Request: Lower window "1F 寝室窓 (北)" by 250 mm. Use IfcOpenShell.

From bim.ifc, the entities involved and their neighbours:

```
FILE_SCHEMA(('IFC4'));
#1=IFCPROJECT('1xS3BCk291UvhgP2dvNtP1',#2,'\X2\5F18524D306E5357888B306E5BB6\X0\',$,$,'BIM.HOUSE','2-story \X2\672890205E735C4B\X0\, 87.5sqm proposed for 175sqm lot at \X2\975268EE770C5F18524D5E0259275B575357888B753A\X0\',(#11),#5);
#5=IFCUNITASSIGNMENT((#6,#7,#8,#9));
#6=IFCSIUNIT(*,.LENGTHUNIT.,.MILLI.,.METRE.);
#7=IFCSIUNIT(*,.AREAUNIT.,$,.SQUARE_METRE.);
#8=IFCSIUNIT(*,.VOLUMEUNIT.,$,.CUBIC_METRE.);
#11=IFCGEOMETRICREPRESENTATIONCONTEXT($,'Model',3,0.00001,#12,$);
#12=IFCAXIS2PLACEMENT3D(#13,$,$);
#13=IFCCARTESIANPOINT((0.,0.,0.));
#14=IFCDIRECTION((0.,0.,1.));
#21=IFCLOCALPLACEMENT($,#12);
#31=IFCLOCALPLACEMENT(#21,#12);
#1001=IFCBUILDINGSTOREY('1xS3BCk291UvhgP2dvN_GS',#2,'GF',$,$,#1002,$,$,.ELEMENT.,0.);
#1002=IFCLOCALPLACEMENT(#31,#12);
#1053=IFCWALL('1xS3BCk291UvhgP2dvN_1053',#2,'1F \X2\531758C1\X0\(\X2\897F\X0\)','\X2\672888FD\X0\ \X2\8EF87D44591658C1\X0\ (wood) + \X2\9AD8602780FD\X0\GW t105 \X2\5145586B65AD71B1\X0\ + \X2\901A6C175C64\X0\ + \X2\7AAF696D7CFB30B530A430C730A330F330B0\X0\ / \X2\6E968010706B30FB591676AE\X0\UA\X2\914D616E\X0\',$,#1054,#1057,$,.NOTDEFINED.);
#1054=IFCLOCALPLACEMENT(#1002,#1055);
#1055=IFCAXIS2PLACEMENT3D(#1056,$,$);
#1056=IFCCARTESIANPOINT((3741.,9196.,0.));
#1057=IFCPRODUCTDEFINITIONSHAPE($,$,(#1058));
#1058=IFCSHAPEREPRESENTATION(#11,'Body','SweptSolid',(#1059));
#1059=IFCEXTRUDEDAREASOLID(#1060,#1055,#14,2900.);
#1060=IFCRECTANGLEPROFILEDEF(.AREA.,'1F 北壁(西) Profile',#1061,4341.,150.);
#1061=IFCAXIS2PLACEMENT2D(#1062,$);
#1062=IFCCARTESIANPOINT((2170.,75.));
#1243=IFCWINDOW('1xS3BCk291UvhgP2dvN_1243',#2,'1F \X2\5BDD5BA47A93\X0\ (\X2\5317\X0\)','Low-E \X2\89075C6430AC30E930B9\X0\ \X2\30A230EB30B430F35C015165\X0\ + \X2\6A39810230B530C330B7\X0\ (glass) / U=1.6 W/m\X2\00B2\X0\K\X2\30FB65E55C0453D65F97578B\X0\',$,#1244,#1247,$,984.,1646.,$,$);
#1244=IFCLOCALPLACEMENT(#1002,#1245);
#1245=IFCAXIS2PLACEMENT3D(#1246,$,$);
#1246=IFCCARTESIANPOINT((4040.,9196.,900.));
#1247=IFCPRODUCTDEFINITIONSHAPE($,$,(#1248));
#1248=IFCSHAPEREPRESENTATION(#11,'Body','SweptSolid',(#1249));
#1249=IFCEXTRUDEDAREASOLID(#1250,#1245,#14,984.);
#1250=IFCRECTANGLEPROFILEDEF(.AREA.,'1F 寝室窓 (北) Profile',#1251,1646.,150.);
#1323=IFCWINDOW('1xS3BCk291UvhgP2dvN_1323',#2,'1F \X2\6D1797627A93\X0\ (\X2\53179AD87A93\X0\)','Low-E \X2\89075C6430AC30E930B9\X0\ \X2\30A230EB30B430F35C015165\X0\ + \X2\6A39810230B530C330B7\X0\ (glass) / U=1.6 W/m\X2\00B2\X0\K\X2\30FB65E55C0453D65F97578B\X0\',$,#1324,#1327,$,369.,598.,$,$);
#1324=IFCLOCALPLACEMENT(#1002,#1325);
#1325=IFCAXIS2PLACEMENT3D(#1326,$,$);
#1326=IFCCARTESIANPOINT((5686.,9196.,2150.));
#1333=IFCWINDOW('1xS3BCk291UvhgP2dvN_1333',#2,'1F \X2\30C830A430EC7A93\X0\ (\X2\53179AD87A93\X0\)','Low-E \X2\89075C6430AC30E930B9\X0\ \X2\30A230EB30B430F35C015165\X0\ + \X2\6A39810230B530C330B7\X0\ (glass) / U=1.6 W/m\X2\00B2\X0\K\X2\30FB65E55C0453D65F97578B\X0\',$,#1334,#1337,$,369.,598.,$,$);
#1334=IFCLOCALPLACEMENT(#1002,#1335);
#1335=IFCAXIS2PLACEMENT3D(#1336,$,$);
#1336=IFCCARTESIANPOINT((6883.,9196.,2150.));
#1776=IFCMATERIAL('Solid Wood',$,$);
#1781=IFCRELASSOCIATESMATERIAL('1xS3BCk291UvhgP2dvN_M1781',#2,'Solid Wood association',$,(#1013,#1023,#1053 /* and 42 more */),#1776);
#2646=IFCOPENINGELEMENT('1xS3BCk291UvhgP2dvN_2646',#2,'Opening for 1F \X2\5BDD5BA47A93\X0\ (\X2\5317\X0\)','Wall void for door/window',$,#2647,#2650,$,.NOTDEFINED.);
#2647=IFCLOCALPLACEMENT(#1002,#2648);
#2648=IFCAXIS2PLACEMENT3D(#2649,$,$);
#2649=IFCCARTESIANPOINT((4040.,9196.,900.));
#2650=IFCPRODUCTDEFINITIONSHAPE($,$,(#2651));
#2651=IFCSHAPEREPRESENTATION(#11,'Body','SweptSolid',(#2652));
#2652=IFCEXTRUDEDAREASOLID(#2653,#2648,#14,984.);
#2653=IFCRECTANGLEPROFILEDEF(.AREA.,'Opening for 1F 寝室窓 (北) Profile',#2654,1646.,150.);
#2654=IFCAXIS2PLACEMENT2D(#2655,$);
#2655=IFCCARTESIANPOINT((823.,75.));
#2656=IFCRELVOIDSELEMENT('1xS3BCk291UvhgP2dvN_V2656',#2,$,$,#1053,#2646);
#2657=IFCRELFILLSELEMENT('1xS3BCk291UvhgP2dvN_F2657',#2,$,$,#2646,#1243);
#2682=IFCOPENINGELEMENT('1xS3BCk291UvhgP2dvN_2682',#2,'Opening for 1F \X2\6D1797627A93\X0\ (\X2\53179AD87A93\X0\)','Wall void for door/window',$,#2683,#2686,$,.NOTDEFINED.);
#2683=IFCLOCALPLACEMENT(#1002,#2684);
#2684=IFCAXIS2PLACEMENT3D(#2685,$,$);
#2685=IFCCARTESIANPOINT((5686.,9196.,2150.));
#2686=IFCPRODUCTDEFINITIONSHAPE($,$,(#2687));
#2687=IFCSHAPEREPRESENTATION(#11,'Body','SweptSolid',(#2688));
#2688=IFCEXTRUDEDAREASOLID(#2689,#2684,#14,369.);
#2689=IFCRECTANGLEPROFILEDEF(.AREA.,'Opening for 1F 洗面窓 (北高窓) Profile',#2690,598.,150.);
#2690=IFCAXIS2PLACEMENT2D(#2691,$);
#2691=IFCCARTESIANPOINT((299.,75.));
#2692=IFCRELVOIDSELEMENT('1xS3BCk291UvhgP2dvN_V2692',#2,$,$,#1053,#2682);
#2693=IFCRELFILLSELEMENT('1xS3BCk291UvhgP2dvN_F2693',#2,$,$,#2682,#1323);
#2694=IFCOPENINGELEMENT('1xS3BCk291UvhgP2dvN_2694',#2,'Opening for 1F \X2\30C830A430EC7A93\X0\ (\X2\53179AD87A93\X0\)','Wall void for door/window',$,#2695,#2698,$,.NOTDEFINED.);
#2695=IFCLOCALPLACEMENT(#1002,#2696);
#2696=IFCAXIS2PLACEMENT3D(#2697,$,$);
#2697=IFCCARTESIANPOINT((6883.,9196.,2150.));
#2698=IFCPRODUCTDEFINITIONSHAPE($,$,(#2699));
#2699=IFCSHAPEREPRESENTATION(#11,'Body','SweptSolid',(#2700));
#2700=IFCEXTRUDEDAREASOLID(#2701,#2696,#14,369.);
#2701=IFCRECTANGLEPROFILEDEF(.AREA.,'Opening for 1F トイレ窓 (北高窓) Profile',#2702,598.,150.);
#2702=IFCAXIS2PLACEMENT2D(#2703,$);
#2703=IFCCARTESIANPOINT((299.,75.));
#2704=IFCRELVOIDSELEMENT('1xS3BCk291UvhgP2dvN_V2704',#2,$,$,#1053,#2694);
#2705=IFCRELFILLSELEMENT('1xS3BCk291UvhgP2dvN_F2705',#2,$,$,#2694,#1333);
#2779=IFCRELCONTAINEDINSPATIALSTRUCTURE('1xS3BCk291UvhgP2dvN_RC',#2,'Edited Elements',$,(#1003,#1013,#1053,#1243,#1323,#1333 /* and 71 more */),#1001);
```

```python
import numpy as np
import ifcopenshell
import ifcopenshell.api.geometry
import ifcopenshell.util.placement
import ifcopenshell.util.unit

model = ifcopenshell.open("bim.ifc")
unit_scale = ifcopenshell.util.unit.calculate_unit_scale(model)

window = model.by_guid("1xS3BCk291UvhgP2dvN_1243")
opening = window.FillsVoids[0].RelatingOpeningElement
dz = -0.25 / unit_scale

shift = np.array([0.0, 0.0, dz])
# The window is not placed relative to its opening, so move both.
for product in (opening, window):
    matrix = ifcopenshell.util.placement.get_local_placement(product.ObjectPlacement)
    matrix[:3, 3] += shift
    ifcopenshell.api.geometry.edit_object_placement(model, product=product, matrix=matrix, is_si=False)

print(f"moved by {dz * unit_scale:+.3f} m")

model.write("bim_v2.ifc")
```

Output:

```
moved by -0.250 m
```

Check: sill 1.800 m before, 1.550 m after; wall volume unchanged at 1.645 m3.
